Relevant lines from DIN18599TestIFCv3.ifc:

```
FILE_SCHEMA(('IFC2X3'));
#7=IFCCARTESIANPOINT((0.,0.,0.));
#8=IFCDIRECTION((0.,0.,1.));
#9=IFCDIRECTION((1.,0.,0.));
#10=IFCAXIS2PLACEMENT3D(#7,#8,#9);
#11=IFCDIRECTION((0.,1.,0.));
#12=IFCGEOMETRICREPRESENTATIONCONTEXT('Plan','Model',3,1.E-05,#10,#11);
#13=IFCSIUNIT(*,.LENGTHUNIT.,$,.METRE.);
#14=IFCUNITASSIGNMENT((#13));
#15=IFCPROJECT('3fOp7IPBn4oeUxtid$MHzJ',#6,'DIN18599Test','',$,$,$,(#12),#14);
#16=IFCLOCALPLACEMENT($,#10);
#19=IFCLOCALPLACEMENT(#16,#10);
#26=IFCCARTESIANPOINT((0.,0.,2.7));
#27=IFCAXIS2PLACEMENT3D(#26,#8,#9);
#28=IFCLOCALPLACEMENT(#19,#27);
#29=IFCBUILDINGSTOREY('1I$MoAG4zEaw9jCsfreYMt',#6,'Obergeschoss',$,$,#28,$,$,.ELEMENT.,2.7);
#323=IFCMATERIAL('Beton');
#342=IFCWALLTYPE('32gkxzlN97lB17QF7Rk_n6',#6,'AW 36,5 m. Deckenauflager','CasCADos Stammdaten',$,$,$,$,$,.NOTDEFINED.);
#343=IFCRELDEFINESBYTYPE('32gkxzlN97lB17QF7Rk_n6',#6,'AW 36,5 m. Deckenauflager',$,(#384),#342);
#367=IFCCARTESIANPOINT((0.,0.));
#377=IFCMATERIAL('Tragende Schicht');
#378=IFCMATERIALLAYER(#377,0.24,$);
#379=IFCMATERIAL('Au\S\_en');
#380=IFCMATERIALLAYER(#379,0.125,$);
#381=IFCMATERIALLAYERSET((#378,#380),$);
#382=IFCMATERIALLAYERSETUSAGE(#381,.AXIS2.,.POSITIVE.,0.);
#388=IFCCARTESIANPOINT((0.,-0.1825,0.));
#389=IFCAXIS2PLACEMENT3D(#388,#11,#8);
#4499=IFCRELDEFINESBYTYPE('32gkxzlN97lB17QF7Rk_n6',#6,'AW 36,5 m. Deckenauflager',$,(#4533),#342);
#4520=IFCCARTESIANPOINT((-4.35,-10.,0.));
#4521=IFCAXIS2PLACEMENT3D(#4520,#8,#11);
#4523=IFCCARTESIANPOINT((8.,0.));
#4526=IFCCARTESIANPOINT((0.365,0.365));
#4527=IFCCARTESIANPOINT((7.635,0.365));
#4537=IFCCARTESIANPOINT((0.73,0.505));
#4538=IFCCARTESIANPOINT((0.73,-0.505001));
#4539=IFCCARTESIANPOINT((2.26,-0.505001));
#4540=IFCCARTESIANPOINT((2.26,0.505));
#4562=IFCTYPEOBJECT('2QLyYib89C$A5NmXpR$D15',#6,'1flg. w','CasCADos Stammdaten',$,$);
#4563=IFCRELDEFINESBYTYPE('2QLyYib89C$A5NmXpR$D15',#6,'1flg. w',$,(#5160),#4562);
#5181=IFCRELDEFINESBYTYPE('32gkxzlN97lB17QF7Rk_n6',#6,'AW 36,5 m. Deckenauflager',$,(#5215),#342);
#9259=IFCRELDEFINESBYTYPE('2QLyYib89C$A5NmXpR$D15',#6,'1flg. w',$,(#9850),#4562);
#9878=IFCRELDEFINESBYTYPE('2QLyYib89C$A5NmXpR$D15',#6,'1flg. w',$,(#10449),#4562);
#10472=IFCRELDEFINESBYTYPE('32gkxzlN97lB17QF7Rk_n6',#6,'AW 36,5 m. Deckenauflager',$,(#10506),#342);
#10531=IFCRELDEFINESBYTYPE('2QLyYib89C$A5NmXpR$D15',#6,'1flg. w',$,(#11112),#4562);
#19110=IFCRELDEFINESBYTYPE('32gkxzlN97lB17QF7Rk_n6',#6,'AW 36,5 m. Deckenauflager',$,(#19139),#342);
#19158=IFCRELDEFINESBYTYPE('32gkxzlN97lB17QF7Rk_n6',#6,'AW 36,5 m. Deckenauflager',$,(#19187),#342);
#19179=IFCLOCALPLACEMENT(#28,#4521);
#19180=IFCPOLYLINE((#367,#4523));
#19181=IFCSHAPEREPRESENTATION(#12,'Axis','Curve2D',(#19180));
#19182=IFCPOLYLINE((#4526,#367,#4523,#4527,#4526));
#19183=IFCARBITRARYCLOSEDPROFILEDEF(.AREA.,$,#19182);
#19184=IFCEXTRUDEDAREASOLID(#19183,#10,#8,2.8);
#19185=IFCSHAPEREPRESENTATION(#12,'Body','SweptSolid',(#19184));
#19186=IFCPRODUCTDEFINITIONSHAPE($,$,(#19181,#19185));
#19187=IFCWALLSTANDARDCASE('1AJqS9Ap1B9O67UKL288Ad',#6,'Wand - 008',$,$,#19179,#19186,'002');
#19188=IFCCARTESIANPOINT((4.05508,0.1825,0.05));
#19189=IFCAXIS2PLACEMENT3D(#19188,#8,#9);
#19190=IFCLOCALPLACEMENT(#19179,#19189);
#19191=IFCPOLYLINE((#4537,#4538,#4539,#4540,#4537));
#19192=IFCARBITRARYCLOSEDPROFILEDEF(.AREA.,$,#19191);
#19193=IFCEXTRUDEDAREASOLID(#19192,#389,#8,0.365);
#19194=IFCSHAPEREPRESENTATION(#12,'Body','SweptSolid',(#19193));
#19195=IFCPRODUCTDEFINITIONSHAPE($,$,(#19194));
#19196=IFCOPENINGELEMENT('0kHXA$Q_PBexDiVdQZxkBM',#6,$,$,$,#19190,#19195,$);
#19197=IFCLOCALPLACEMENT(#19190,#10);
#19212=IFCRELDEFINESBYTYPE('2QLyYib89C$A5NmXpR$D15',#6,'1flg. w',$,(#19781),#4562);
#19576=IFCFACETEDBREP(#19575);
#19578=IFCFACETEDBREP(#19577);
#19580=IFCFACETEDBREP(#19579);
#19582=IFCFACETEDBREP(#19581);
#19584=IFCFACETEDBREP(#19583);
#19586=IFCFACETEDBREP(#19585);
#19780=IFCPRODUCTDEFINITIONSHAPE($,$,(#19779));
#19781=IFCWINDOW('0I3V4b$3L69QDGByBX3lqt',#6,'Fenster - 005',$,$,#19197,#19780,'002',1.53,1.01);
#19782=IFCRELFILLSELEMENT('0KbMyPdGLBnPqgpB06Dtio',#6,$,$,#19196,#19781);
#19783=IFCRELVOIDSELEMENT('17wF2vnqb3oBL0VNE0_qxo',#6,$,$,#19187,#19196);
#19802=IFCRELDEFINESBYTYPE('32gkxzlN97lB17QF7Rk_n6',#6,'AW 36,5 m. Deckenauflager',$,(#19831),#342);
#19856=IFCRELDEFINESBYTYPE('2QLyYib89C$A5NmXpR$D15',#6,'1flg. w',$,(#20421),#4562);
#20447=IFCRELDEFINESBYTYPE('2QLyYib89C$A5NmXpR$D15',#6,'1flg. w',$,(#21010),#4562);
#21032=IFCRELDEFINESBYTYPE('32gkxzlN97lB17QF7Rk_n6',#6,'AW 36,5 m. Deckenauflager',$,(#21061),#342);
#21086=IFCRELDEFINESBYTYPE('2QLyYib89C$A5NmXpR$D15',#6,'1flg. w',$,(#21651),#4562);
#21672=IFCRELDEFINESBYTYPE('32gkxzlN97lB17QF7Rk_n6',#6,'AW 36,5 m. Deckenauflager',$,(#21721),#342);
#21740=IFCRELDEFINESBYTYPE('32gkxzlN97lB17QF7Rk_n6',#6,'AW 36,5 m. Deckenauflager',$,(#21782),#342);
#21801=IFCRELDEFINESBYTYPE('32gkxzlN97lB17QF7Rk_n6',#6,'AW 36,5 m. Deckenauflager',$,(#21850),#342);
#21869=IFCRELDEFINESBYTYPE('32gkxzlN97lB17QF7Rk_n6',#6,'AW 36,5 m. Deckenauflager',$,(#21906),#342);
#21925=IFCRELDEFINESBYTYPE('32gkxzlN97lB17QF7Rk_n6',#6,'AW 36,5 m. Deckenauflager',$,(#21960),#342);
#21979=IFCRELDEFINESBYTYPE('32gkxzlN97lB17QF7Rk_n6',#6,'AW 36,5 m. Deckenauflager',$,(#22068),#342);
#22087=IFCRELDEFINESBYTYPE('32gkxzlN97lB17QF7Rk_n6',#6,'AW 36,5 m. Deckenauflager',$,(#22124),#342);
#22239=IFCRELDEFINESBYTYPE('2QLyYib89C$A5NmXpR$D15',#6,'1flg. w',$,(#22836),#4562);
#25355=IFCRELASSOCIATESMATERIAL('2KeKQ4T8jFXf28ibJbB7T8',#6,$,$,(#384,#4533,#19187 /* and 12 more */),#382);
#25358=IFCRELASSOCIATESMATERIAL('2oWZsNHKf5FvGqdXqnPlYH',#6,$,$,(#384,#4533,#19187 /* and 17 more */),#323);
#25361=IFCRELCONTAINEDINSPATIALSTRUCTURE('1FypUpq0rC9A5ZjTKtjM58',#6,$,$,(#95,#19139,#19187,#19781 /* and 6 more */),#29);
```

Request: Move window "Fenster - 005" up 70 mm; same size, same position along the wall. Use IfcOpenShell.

```python
import numpy as np
import ifcopenshell
import ifcopenshell.api.geometry
import ifcopenshell.util.placement
import ifcopenshell.util.unit

model = ifcopenshell.open("DIN18599TestIFCv3.ifc")
unit_scale = ifcopenshell.util.unit.calculate_unit_scale(model)

window = model.by_id(19781)
opening = window.FillsVoids[0].RelatingOpeningElement
dz = 0.07 / unit_scale

shift = np.array([0.0, 0.0, dz])
# The window is placed relative to its opening, so it follows when the opening moves.
matrix = ifcopenshell.util.placement.get_local_placement(opening.ObjectPlacement)
matrix[:3, 3] += shift
ifcopenshell.api.geometry.edit_object_placement(
    model, product=opening, matrix=matrix, is_si=False, should_transform_children=True
)

print(f"moved by {dz * unit_scale:+.3f} m")

model.write("DIN18599TestIFCv3_edited.ifc")
```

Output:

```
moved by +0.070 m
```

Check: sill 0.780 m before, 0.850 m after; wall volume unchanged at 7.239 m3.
